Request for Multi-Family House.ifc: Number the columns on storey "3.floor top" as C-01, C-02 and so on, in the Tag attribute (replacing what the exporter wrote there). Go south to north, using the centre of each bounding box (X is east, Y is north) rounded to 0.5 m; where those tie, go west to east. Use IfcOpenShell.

First a look at what the model holds.

```python
import ifcopenshell
import ifcopenshell.util.element
import ifcopenshell.util.placement

model = ifcopenshell.open("Multi-Family House.ifc")
print(model.schema)
storey = next(s for s in model.by_type("IfcBuildingStorey") if s.Name == "3.floor top")
columns = [e for e in ifcopenshell.util.element.get_decomposition(storey) if e.is_a("IfcColumn")]
for e in sorted(columns, key=lambda e: e.id()):
    origin = ifcopenshell.util.placement.get_local_placement(e.ObjectPlacement)[:3, 3]
    print(e.id(), e.Tag, e.Name, origin.round(2) + 0.0, sep=" | ")
```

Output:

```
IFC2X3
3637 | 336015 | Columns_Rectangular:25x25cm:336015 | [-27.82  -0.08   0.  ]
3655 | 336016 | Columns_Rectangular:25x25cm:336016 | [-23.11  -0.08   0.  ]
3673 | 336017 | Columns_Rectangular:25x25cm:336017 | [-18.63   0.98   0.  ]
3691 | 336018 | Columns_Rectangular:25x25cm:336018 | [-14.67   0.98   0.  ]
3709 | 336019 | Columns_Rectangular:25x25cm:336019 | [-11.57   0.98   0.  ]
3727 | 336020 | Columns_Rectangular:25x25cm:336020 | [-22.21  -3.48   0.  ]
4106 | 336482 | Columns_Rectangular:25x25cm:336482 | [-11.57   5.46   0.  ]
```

```python
import ifcopenshell
import ifcopenshell.geom
import ifcopenshell.util.element
import ifcopenshell.util.shape

model = ifcopenshell.open("Multi-Family House.ifc")
settings = ifcopenshell.geom.settings()
settings.set("use-world-coords", True)


def centre(element):
    shape = ifcopenshell.geom.create_shape(settings, element)
    return ifcopenshell.util.shape.get_bbox_centroid(shape.geometry)


storey = next(s for s in model.by_type("IfcBuildingStorey") if s.Name == "3.floor top")
columns = [e for e in ifcopenshell.util.element.get_decomposition(storey) if e.is_a("IfcColumn")]

# Insertion points can sit at a corner or the storey origin, so sort by the geometry (in metres).
centres = {e: centre(e) for e in columns}
columns.sort(key=lambda e: (round(centres[e][1] / 0.5), centres[e][0]))

for i, e in enumerate(columns, start=1):
    number = f"C-{i:02d}"
    e.Tag = number
    print(e.id(), number)

model.write("Multi-Family House_updated.ifc")
```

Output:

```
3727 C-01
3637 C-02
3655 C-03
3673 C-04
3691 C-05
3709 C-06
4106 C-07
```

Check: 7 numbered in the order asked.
